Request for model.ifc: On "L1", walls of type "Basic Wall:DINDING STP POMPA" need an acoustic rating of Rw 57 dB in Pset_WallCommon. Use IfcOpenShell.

First a look at what the model holds.

```python
import ifcopenshell
import ifcopenshell.util.element

model = ifcopenshell.open("model.ifc")
print(model.schema)
storey = next(s for s in model.by_type("IfcBuildingStorey") if s.Name == "L1")
walls = [e for e in ifcopenshell.util.element.get_decomposition(storey) if e.is_a("IfcWall")]
seen = {}
for e in walls:
    element_type = ifcopenshell.util.element.get_type(e)
    key = (element_type.Name if element_type != e and element_type else None, ifcopenshell.util.element.get_pset(e, "Pset_WallCommon", "AcousticRating"))
    seen[key] = seen.get(key, 0) + 1
for (name, value), count in sorted(seen.items(), key=str):
    print(count, "x", name, "|", value)
```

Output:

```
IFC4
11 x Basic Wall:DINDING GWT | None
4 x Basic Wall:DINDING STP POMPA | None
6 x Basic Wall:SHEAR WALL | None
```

```python
import ifcopenshell
import ifcopenshell.api.pset
import ifcopenshell.util.element

model = ifcopenshell.open("model.ifc")

storey = next(s for s in model.by_type("IfcBuildingStorey") if s.Name == "L1")
walls = [e for e in ifcopenshell.util.element.get_decomposition(storey) if e.is_a("IfcWall")]

count = 0
for e in walls:
    element_type = ifcopenshell.util.element.get_type(e)
    if element_type in (None, e) or element_type.Name != "Basic Wall:DINDING STP POMPA":
        continue
    # add_pset returns the element's existing set when there is one.
    pset = ifcopenshell.api.pset.add_pset(model, product=e, name="Pset_WallCommon")
    ifcopenshell.api.pset.edit_pset(model, pset=pset, properties={"AcousticRating": "Rw 57 dB"})
    count += 1

print(count, "walls updated")

model.write("model_v2.ifc")
```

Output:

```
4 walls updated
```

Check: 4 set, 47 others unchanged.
